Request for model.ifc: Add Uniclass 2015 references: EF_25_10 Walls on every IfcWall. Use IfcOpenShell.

First a look at what the model holds.

```python
import ifcopenshell

model = ifcopenshell.open("model.ifc")
print(model.schema)
print("classifications:", [c.Name for c in model.by_type("IfcClassification")])
for ifc_class in ("IfcDoor", "IfcRoof", "IfcStair", "IfcWall", "IfcWindow"):
    print(ifc_class, len(model.by_type(ifc_class)))
```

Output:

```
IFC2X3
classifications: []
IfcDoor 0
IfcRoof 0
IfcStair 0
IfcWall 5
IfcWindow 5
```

```python
import ifcopenshell
import ifcopenshell.api.classification

model = ifcopenshell.open("model.ifc")

# IFC2X3 requires Source and Edition and has no link from the project to the system.
system = model.create_entity("IfcClassification", Source="NBS", Edition="2015", Name="Uniclass 2015")

codes = {
    "IfcWall": ("EF_25_10", "Walls"),
}
for ifc_class, (code, name) in codes.items():
    products = model.by_type(ifc_class)
    ifcopenshell.api.classification.add_reference(
        model, products=products, classification=system, identification=code, name=name
    )
    print(code, len(products))

model.write("model_rev.ifc")
```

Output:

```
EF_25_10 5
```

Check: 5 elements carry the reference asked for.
